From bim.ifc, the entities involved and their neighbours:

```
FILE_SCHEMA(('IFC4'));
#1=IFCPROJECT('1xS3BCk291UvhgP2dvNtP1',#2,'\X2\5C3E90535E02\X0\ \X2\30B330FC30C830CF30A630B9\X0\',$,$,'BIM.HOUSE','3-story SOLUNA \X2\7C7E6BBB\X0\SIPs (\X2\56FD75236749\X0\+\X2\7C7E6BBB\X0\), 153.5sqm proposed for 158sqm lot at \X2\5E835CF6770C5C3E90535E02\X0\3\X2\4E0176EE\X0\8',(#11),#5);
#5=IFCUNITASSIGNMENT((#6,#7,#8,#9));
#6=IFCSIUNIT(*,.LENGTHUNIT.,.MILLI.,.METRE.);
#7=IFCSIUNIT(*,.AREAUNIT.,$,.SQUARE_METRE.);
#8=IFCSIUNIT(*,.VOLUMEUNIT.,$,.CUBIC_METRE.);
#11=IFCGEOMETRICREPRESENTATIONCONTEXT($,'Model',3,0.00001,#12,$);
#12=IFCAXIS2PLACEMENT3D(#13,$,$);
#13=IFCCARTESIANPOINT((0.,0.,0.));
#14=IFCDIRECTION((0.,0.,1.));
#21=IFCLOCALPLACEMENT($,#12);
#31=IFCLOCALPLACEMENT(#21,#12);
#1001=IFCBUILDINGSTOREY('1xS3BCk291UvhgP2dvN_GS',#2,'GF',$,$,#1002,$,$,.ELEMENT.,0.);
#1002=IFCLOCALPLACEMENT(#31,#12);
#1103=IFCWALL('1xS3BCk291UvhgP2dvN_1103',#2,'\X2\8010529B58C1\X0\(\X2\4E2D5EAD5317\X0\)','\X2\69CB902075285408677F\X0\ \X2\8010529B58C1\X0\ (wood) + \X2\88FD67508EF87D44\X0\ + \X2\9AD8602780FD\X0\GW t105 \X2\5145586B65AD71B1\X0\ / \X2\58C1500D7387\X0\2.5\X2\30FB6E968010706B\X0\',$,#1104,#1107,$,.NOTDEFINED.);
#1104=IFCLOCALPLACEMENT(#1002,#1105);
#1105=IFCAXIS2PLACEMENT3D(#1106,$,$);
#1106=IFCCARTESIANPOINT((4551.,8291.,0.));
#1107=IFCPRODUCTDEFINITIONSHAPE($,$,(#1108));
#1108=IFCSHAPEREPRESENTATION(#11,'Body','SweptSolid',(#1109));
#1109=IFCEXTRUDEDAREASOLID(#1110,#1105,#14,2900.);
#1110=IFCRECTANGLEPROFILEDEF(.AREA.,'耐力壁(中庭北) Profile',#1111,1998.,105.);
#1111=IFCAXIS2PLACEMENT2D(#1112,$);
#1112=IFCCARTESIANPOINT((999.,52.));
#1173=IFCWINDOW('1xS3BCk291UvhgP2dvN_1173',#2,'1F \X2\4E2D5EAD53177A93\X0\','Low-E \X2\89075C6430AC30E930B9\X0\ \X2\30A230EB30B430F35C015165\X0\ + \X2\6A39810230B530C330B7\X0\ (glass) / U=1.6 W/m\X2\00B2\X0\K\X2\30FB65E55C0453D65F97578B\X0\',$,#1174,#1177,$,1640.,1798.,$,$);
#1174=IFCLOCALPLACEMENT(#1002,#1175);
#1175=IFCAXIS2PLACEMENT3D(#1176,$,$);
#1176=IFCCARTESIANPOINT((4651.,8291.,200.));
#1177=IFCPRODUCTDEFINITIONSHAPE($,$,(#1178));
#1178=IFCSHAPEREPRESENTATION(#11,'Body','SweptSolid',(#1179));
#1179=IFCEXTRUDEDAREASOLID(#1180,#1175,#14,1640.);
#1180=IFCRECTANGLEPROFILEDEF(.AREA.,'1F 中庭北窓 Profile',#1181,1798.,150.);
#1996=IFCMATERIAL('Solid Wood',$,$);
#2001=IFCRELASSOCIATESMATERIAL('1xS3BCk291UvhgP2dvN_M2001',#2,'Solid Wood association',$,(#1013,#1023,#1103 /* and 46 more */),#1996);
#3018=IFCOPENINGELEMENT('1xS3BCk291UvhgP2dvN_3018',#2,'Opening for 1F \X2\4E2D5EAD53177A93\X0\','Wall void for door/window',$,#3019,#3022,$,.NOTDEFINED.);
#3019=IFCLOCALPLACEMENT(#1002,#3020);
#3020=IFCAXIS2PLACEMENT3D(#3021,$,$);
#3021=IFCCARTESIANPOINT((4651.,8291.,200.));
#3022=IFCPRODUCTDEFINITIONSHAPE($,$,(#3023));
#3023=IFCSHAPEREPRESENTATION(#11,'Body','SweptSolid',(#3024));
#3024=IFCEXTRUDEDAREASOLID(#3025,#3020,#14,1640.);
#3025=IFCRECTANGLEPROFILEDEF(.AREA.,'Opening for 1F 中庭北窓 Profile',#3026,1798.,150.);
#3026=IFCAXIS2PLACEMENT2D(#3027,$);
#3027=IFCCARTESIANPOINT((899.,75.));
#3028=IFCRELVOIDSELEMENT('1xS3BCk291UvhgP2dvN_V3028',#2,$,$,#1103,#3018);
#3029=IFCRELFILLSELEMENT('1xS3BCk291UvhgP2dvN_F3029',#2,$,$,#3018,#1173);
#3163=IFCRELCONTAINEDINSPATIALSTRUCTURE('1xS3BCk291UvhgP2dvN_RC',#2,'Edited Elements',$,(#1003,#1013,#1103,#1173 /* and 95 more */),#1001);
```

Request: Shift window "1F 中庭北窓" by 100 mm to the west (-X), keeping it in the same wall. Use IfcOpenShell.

```python
import ifcopenshell
import ifcopenshell.api.geometry
import ifcopenshell.util.placement
import ifcopenshell.util.unit

model = ifcopenshell.open("bim.ifc")
unit_scale = ifcopenshell.util.unit.calculate_unit_scale(model)

window = model.by_id(1173)
opening = window.FillsVoids[0].RelatingOpeningElement
wall = opening.VoidsElements[0].RelatingBuildingElement

wall_matrix = ifcopenshell.util.placement.get_local_placement(wall.ObjectPlacement)
shift = wall_matrix[:3, 0] * -0.1 / unit_scale
before = ifcopenshell.util.placement.get_local_placement(window.ObjectPlacement)[:3, 3].copy()

# The window is not placed relative to its opening, so move both.
for product in (opening, window):
    matrix = ifcopenshell.util.placement.get_local_placement(product.ObjectPlacement)
    matrix[:3, 3] += shift
    ifcopenshell.api.geometry.edit_object_placement(model, product=product, matrix=matrix, is_si=False)

after = ifcopenshell.util.placement.get_local_placement(window.ObjectPlacement)[:3, 3]
print("window moved by", (after - before).round(3) + 0.0)

model.write("bim_v2.ifc")
```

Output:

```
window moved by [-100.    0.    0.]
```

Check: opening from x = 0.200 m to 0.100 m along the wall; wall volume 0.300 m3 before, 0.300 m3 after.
